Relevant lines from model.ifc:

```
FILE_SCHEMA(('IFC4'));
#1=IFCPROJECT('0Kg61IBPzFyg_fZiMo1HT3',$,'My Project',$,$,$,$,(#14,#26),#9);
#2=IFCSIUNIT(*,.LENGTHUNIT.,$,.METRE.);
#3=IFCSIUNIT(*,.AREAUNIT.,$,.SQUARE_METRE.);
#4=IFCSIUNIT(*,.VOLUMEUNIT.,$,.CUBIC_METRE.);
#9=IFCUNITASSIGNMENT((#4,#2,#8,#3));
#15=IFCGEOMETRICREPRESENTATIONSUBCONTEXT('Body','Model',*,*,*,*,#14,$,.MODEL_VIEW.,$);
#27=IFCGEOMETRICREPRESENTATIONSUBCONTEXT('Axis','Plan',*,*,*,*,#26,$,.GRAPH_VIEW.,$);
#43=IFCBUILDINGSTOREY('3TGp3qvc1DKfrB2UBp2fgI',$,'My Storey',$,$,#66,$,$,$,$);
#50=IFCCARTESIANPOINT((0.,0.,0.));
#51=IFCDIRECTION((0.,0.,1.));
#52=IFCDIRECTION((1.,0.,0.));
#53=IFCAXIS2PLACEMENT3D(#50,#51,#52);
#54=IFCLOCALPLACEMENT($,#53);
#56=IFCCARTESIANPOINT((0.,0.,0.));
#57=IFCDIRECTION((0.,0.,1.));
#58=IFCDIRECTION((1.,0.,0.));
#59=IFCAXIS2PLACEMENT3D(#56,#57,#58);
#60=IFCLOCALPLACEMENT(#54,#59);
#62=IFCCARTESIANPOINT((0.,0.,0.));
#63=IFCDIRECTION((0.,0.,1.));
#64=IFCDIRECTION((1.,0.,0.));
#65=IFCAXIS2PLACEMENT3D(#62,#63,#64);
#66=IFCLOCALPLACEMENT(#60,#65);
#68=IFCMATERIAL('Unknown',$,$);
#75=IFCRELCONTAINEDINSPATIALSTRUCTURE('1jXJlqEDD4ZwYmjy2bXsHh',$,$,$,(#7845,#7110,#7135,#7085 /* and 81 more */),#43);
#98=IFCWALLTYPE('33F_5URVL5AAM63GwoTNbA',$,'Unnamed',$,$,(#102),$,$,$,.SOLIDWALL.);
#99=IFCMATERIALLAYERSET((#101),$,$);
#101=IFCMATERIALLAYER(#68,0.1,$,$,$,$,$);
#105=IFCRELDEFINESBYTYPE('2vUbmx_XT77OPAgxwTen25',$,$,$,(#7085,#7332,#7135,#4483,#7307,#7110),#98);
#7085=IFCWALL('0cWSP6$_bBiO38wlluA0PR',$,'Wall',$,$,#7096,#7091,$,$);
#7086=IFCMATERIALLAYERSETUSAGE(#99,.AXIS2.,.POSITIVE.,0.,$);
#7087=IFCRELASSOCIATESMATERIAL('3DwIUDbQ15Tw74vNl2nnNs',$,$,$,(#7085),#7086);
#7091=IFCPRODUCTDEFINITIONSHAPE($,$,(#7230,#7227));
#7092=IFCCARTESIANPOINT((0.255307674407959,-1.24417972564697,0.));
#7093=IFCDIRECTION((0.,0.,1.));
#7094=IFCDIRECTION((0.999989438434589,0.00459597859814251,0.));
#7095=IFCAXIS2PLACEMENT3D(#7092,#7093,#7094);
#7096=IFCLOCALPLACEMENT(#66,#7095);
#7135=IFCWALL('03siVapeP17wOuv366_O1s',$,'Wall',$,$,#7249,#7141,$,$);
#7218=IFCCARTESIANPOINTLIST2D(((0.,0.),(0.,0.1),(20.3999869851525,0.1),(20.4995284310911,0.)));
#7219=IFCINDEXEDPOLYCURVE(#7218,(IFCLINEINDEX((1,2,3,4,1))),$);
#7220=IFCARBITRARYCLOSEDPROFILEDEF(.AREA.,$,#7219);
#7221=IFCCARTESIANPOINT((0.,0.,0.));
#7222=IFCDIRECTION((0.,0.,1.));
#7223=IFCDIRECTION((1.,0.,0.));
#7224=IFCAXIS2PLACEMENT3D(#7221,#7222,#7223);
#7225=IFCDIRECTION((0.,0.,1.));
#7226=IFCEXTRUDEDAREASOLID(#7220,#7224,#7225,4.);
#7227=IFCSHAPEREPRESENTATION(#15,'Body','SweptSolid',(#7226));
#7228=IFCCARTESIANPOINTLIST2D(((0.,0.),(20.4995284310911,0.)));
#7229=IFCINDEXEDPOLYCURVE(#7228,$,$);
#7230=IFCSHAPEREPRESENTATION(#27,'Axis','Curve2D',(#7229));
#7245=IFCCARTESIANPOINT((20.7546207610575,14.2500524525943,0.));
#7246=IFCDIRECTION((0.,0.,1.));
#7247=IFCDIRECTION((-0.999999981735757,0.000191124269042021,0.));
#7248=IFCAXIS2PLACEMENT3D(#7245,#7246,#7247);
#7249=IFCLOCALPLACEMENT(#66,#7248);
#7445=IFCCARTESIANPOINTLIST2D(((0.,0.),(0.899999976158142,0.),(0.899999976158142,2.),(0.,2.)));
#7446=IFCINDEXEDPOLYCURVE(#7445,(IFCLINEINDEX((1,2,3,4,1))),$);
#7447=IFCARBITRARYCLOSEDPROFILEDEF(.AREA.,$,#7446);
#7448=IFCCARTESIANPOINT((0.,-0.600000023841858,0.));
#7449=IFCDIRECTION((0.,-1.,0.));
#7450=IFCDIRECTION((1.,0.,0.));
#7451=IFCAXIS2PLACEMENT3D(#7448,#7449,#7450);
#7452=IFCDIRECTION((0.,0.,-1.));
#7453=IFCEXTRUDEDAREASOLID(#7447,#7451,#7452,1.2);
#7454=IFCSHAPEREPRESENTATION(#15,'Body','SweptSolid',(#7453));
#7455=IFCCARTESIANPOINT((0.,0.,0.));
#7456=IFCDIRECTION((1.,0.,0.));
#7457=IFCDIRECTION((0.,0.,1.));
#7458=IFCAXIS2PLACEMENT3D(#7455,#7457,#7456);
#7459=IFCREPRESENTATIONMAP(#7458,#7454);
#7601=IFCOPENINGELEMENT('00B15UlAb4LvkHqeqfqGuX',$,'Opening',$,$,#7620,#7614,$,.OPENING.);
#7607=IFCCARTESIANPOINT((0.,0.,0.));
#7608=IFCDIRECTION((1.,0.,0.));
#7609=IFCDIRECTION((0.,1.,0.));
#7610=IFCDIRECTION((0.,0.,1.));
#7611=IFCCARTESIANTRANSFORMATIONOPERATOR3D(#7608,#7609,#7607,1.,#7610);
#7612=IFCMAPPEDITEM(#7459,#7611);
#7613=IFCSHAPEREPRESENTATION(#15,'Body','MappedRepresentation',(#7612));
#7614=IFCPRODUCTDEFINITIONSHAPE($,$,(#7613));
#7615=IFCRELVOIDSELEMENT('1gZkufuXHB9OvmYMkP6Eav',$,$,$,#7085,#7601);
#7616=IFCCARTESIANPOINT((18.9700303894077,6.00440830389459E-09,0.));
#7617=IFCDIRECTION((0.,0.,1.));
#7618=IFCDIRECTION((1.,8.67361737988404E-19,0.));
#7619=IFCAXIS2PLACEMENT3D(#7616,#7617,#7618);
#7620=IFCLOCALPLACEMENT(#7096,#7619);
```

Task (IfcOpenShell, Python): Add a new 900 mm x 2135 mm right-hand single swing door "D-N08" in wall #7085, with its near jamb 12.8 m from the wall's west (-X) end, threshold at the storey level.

```python
import numpy as np
import ifcopenshell
import ifcopenshell.api.feature
import ifcopenshell.api.geometry
import ifcopenshell.api.root
import ifcopenshell.api.spatial
import ifcopenshell.geom
import ifcopenshell.util.element
import ifcopenshell.util.placement
import ifcopenshell.util.representation
import ifcopenshell.util.shape
import ifcopenshell.util.unit

model = ifcopenshell.open("model.ifc")
unit_scale = ifcopenshell.util.unit.calculate_unit_scale(model)
settings = ifcopenshell.geom.settings()


def volume(element):
    """Net volume in cubic metres, openings subtracted."""
    shape = ifcopenshell.geom.create_shape(settings, element)
    return ifcopenshell.util.shape.get_volume(shape.geometry)


wall = model.by_id(7085)
storey = ifcopenshell.util.element.get_container(wall, ifc_class="IfcBuildingStorey")
context = ifcopenshell.util.representation.get_context(model, "Model", "Body", "MODEL_VIEW")
before = volume(wall)

width, height, from_end, sill = 0.9, 2.135, 12.8, 0.0  # metres

# The wall runs along its own X axis, and the end named is its -X end.
wall_shape = ifcopenshell.geom.create_shape(settings, wall)
x, y, z = ifcopenshell.util.shape.get_vertices(wall_shape.geometry).T
start = x.min() + from_end
face, thickness = float(y.min()), float(y.max() - y.min())
wall_matrix = ifcopenshell.util.placement.get_local_placement(wall.ObjectPlacement)
level = ifcopenshell.util.placement.get_local_placement(storey.ObjectPlacement)[2, 3]


def in_wall(x, y):
    """Placement at x, y metres in the wall's axes, at sill height."""
    matrix = wall_matrix.copy()
    matrix[:, 3] = wall_matrix @ np.array([x / unit_scale, y / unit_scale, 0.0, 1.0])
    matrix[2, 3] = level + sill / unit_scale
    return matrix


# Opening: a box that overshoots both wall faces by 50 mm.
opening = ifcopenshell.api.root.create_entity(model, ifc_class="IfcOpeningElement", predefined_type="OPENING")
box = ifcopenshell.api.geometry.add_wall_representation(
    model, context=context, length=width, height=height, thickness=thickness + 0.1
)
ifcopenshell.api.geometry.assign_representation(model, product=opening, representation=box)
ifcopenshell.api.geometry.edit_object_placement(model, product=opening, matrix=in_wall(start, face - 0.05), is_si=False)
ifcopenshell.api.feature.add_feature(model, feature=opening, element=wall)

door = ifcopenshell.api.root.create_entity(model, ifc_class="IfcDoor", name="D-N08", predefined_type="DOOR")
door.OverallWidth, door.OverallHeight = width / unit_scale, height / unit_scale
door.OperationType = "SINGLE_SWING_RIGHT"
body = ifcopenshell.api.geometry.add_door_representation(
    model,
    context=context,
    overall_width=door.OverallWidth,
    overall_height=door.OverallHeight,
    operation_type="SINGLE_SWING_RIGHT",
    lining_properties={"LiningDepth": thickness / unit_scale, "ThresholdDepth": thickness / unit_scale},
)
ifcopenshell.api.geometry.assign_representation(model, product=door, representation=body)
ifcopenshell.api.spatial.assign_container(model, products=[door], relating_structure=storey)
ifcopenshell.api.feature.add_filling(model, opening=opening, element=door)

# The lining spans the wall, so the door starts at the wall face.
ifcopenshell.api.geometry.edit_object_placement(model, product=door, matrix=in_wall(start, face), is_si=False)

after = volume(wall)

print(f"wall volume {before:.3f} -> {after:.3f} m3")

model.write("model_rev.ifc")
```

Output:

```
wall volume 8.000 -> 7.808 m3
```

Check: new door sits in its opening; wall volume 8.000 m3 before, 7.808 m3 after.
